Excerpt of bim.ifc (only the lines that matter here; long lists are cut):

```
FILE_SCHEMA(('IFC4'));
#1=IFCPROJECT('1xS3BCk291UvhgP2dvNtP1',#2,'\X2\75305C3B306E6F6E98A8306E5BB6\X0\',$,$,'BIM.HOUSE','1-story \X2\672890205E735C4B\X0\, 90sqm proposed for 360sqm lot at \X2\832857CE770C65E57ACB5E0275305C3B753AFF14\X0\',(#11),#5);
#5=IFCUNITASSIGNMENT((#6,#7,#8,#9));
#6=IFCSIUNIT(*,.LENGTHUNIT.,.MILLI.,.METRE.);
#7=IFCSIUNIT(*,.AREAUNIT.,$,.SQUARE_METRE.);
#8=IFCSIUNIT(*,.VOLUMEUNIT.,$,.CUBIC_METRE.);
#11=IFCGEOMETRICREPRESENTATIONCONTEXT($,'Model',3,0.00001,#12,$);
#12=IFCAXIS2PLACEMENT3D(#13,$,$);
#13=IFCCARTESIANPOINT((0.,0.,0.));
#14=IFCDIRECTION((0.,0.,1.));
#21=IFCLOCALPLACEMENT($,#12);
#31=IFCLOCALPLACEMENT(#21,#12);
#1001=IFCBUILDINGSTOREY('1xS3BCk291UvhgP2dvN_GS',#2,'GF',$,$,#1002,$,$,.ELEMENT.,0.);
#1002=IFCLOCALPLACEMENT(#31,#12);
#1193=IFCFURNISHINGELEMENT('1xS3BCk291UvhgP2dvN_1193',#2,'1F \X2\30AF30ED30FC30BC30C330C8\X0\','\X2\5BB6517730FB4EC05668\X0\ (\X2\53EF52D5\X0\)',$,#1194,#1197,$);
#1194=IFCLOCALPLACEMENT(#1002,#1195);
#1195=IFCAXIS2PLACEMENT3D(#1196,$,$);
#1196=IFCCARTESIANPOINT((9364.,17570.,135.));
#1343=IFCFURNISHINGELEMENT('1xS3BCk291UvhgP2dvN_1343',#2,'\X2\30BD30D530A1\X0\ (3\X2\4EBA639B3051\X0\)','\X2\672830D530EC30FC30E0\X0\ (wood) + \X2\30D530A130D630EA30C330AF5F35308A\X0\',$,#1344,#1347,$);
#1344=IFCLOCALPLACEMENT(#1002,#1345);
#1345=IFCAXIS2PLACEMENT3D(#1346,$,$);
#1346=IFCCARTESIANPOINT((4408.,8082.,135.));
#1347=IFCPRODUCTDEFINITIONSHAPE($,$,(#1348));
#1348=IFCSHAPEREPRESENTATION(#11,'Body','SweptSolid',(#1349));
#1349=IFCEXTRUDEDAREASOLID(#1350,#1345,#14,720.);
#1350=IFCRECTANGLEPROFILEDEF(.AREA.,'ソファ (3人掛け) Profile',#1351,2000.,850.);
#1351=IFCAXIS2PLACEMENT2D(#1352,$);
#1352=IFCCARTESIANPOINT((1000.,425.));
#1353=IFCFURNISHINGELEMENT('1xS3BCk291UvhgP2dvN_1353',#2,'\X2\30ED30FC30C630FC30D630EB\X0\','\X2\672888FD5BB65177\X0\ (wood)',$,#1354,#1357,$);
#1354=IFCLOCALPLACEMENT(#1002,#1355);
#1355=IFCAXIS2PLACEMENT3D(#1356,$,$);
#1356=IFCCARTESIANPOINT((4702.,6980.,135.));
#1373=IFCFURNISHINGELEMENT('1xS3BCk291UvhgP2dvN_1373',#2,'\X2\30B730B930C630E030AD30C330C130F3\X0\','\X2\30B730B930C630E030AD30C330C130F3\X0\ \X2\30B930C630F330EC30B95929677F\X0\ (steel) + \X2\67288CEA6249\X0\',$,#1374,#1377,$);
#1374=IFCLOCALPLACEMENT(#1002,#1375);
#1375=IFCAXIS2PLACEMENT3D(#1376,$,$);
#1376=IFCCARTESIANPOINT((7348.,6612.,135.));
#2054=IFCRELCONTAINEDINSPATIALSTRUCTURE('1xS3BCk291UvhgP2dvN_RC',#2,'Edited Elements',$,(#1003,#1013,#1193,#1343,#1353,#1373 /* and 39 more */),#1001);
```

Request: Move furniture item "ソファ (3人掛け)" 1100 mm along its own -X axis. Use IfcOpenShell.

```python
import ifcopenshell
import ifcopenshell.api.geometry
import ifcopenshell.util.placement
import ifcopenshell.util.unit

model = ifcopenshell.open("bim.ifc")
unit_scale = ifcopenshell.util.unit.calculate_unit_scale(model)

item = model.by_id(1343)
matrix = ifcopenshell.util.placement.get_local_placement(item.ObjectPlacement)
matrix[:3, 3] -= matrix[:3, 0] * 1.1 / unit_scale
ifcopenshell.api.geometry.edit_object_placement(model, product=item, matrix=matrix, is_si=False)

print(ifcopenshell.util.placement.get_local_placement(item.ObjectPlacement).round(3) + 0.0)

model.write("bim_updated.ifc")
```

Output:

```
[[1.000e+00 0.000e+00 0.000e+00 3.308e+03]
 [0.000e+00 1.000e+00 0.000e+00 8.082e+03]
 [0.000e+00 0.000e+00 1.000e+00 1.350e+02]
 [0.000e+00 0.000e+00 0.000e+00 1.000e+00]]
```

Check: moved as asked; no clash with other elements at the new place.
